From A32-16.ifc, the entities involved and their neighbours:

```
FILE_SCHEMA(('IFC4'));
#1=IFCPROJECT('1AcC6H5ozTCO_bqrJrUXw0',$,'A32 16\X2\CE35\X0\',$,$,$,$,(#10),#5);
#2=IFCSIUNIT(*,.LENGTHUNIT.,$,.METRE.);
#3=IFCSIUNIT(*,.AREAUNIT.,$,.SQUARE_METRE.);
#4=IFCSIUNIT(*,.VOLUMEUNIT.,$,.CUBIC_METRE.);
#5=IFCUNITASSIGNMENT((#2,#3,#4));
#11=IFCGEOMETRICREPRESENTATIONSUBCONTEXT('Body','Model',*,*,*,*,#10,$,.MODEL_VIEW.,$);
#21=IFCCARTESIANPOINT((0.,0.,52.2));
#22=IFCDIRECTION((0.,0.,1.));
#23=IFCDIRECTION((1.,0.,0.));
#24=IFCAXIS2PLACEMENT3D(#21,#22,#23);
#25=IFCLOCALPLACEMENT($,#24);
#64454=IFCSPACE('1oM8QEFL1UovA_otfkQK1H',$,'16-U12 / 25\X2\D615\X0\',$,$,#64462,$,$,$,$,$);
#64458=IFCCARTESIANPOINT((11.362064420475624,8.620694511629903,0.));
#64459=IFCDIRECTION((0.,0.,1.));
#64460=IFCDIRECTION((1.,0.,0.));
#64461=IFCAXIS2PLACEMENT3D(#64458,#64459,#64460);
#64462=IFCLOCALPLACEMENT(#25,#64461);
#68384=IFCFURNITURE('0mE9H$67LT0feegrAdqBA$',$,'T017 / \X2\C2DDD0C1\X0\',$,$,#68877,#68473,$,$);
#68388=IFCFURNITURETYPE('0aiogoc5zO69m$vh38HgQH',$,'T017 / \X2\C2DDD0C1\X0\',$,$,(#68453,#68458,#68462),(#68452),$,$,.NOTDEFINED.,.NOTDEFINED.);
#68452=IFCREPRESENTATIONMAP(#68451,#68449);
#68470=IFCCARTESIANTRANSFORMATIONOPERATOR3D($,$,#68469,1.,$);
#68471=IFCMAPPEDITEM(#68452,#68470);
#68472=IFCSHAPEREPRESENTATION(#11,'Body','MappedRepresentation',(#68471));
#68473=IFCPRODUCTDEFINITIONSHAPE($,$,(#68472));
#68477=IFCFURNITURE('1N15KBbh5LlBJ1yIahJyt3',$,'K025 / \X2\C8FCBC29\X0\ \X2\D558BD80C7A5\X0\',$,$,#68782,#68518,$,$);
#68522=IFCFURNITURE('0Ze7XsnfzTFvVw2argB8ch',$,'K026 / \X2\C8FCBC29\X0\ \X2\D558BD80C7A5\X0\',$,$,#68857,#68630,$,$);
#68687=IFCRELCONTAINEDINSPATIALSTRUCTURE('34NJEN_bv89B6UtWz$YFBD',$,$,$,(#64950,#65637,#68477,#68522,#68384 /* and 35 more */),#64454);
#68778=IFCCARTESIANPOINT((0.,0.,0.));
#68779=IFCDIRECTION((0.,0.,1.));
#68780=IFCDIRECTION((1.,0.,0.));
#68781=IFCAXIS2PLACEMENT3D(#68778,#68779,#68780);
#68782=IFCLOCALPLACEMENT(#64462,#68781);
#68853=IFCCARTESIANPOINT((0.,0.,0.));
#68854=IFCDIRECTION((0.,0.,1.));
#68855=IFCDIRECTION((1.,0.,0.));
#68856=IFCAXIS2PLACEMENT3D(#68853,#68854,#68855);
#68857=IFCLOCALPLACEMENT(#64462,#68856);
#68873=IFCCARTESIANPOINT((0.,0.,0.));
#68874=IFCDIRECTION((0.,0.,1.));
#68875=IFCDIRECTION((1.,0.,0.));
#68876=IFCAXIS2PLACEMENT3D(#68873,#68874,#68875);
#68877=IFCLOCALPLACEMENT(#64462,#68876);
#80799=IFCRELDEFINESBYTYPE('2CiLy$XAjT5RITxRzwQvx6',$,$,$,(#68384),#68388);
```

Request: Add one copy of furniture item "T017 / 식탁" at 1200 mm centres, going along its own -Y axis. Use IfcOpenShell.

```python
import ifcopenshell
import ifcopenshell.api.geometry
import ifcopenshell.api.root
import ifcopenshell.util.element
import ifcopenshell.util.placement

model = ifcopenshell.open("A32-16.ifc")

source = model.by_id(68384)
base = ifcopenshell.util.placement.get_local_placement(source.ObjectPlacement)
step = -base[:3, 1] * 1.2

for i in range(1, 2):
    copy = ifcopenshell.api.root.copy_class(model, product=source)
    copy.Representation = ifcopenshell.util.element.copy_deep(
        model, source.Representation, exclude=["IfcGeometricRepresentationContext", "IfcRepresentationMap"]
    )
    matrix = base.copy()
    matrix[:3, 3] += i * step
    print("added at", matrix[:3, 3].round(3) + 0.0)
    ifcopenshell.api.geometry.edit_object_placement(model, product=copy, matrix=matrix, is_si=False)

model.write("A32-16_v2.ifc")
```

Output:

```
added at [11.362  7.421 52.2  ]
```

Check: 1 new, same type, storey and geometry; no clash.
